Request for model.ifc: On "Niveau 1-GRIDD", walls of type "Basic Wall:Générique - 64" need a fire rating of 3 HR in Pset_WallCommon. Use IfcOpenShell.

First a look at what the model holds.

```python
import ifcopenshell
import ifcopenshell.util.element

model = ifcopenshell.open("model.ifc")
print(model.schema)
storey = next(s for s in model.by_type("IfcBuildingStorey") if s.Name == "Niveau 1-GRIDD")
walls = [e for e in ifcopenshell.util.element.get_decomposition(storey) if e.is_a("IfcWall")]
seen = {}
for e in walls:
    element_type = ifcopenshell.util.element.get_type(e)
    key = (element_type.Name if element_type != e and element_type else None, ifcopenshell.util.element.get_pset(e, "Pset_WallCommon", "FireRating"))
    seen[key] = seen.get(key, 0) + 1
for (name, value), count in sorted(seen.items(), key=str):
    print(count, "x", name, "|", value)
```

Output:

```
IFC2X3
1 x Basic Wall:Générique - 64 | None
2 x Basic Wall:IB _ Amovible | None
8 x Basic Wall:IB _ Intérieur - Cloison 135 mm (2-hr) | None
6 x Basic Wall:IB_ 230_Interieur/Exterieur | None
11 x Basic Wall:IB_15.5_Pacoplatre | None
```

```python
import ifcopenshell
import ifcopenshell.api.pset
import ifcopenshell.util.element

model = ifcopenshell.open("model.ifc")

storey = next(s for s in model.by_type("IfcBuildingStorey") if s.Name == "Niveau 1-GRIDD")
walls = [e for e in ifcopenshell.util.element.get_decomposition(storey) if e.is_a("IfcWall")]

count = 0
for e in walls:
    element_type = ifcopenshell.util.element.get_type(e)
    if element_type in (None, e) or element_type.Name != "Basic Wall:Générique - 64":
        continue
    # add_pset returns the element's existing set when there is one.
    pset = ifcopenshell.api.pset.add_pset(model, product=e, name="Pset_WallCommon")
    ifcopenshell.api.pset.edit_pset(model, pset=pset, properties={"FireRating": "3 HR"})
    count += 1

print(count, "walls updated")

model.write("model-out.ifc")
```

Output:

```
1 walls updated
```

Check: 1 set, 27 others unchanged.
